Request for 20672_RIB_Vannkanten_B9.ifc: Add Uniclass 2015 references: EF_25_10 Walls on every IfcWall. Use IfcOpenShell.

First a look at what the model holds.

```python
import ifcopenshell

model = ifcopenshell.open("20672_RIB_Vannkanten_B9.ifc")
print(model.schema)
print("classifications:", [c.Name for c in model.by_type("IfcClassification")])
for ifc_class in ("IfcDoor", "IfcRoof", "IfcStair", "IfcWall", "IfcWindow"):
    print(ifc_class, len(model.by_type(ifc_class)))
```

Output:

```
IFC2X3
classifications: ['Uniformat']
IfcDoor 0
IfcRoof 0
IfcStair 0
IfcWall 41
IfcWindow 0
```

```python
import ifcopenshell
import ifcopenshell.api.classification

model = ifcopenshell.open("20672_RIB_Vannkanten_B9.ifc")

# IFC2X3 requires Source and Edition and has no link from the project to the system.
system = model.create_entity("IfcClassification", Source="NBS", Edition="2015", Name="Uniclass 2015")

codes = {
    "IfcWall": ("EF_25_10", "Walls"),
}
for ifc_class, (code, name) in codes.items():
    products = model.by_type(ifc_class)
    ifcopenshell.api.classification.add_reference(
        model, products=products, classification=system, identification=code, name=name
    )
    print(code, len(products))

model.write("20672_RIB_Vannkanten_B9_v2.ifc")
```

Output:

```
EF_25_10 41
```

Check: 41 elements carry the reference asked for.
